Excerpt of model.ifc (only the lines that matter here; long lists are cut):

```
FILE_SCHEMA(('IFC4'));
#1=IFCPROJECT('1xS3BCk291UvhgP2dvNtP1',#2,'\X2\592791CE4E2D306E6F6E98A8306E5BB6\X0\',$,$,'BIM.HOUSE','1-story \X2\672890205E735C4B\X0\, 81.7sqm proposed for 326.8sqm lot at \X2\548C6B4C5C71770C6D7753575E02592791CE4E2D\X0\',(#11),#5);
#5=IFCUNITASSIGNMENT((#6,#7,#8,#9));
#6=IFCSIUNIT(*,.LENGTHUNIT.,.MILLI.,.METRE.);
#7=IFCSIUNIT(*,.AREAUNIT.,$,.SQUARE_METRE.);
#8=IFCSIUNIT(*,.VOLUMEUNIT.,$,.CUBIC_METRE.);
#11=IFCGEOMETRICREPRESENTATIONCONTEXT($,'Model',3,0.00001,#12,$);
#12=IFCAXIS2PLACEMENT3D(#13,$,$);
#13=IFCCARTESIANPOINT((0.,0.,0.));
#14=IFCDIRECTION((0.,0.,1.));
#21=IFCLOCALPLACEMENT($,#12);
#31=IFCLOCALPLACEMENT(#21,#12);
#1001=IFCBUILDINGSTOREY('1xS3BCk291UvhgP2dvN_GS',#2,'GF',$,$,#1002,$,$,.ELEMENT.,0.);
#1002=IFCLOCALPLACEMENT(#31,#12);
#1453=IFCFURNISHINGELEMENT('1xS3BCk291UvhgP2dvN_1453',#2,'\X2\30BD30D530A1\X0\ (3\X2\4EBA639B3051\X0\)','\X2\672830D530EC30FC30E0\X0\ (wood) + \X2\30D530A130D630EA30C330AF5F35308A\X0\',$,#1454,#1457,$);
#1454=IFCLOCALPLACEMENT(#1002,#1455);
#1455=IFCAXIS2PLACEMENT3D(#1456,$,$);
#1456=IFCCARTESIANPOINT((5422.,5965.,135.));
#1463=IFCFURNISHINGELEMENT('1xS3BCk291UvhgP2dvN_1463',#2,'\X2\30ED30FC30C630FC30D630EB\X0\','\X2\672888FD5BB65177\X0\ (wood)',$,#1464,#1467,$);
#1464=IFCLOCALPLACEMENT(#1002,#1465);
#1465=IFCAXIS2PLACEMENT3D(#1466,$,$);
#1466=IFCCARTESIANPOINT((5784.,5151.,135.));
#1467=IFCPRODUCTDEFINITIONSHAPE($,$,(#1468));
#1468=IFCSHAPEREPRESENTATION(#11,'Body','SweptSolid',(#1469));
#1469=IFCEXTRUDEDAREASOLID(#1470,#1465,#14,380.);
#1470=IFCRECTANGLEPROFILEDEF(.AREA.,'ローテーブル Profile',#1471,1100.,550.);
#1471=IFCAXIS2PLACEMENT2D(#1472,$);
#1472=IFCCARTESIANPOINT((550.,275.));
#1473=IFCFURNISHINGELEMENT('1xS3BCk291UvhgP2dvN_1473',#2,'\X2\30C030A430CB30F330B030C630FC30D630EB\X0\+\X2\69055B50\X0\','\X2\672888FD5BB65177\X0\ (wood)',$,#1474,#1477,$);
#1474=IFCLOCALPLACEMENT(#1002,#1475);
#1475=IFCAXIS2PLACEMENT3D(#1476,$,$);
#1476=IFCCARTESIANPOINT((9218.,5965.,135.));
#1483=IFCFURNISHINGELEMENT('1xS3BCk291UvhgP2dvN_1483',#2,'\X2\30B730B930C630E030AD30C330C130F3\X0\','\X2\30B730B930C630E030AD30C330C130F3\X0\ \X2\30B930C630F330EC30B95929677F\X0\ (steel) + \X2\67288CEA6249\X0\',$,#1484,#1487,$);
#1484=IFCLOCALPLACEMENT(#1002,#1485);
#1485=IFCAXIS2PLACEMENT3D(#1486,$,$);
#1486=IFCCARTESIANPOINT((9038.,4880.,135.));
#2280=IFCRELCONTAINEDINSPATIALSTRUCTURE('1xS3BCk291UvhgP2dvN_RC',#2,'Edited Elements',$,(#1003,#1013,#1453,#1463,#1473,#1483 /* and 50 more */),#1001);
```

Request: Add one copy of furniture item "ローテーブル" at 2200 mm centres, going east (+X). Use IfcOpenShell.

```python
import numpy as np
import ifcopenshell
import ifcopenshell.api.geometry
import ifcopenshell.api.root
import ifcopenshell.util.element
import ifcopenshell.util.placement
import ifcopenshell.util.unit

model = ifcopenshell.open("model.ifc")
unit_scale = ifcopenshell.util.unit.calculate_unit_scale(model)


def reuse_history(source, copy):
    """copy_class also copies each property set's owner history, people and application; keep the originals."""
    for rel in copy.IsDefinedBy:
        if rel.is_a("IfcRelDefinesByProperties") and (history := rel.RelatingPropertyDefinition.OwnerHistory):
            rel.RelatingPropertyDefinition.OwnerHistory = source.OwnerHistory
            ifcopenshell.util.element.remove_deep2(model, history)


source = model.by_guid("1xS3BCk291UvhgP2dvN_1463")
base = ifcopenshell.util.placement.get_local_placement(source.ObjectPlacement)
step = np.array([1.0, 0.0, 0.0]) * 2.2 / unit_scale

for i in range(1, 2):
    copy = ifcopenshell.api.root.copy_class(model, product=source)
    copy.Representation = ifcopenshell.util.element.copy_deep(
        model, source.Representation, exclude=["IfcGeometricRepresentationContext", "IfcRepresentationMap"]
    )
    reuse_history(source, copy)
    matrix = base.copy()
    matrix[:3, 3] += i * step
    print("added at", matrix[:3, 3].round(3) + 0.0)
    ifcopenshell.api.geometry.edit_object_placement(model, product=copy, matrix=matrix, is_si=False)

model.write("model_updated.ifc")
```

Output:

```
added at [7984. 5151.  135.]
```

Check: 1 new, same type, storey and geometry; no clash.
